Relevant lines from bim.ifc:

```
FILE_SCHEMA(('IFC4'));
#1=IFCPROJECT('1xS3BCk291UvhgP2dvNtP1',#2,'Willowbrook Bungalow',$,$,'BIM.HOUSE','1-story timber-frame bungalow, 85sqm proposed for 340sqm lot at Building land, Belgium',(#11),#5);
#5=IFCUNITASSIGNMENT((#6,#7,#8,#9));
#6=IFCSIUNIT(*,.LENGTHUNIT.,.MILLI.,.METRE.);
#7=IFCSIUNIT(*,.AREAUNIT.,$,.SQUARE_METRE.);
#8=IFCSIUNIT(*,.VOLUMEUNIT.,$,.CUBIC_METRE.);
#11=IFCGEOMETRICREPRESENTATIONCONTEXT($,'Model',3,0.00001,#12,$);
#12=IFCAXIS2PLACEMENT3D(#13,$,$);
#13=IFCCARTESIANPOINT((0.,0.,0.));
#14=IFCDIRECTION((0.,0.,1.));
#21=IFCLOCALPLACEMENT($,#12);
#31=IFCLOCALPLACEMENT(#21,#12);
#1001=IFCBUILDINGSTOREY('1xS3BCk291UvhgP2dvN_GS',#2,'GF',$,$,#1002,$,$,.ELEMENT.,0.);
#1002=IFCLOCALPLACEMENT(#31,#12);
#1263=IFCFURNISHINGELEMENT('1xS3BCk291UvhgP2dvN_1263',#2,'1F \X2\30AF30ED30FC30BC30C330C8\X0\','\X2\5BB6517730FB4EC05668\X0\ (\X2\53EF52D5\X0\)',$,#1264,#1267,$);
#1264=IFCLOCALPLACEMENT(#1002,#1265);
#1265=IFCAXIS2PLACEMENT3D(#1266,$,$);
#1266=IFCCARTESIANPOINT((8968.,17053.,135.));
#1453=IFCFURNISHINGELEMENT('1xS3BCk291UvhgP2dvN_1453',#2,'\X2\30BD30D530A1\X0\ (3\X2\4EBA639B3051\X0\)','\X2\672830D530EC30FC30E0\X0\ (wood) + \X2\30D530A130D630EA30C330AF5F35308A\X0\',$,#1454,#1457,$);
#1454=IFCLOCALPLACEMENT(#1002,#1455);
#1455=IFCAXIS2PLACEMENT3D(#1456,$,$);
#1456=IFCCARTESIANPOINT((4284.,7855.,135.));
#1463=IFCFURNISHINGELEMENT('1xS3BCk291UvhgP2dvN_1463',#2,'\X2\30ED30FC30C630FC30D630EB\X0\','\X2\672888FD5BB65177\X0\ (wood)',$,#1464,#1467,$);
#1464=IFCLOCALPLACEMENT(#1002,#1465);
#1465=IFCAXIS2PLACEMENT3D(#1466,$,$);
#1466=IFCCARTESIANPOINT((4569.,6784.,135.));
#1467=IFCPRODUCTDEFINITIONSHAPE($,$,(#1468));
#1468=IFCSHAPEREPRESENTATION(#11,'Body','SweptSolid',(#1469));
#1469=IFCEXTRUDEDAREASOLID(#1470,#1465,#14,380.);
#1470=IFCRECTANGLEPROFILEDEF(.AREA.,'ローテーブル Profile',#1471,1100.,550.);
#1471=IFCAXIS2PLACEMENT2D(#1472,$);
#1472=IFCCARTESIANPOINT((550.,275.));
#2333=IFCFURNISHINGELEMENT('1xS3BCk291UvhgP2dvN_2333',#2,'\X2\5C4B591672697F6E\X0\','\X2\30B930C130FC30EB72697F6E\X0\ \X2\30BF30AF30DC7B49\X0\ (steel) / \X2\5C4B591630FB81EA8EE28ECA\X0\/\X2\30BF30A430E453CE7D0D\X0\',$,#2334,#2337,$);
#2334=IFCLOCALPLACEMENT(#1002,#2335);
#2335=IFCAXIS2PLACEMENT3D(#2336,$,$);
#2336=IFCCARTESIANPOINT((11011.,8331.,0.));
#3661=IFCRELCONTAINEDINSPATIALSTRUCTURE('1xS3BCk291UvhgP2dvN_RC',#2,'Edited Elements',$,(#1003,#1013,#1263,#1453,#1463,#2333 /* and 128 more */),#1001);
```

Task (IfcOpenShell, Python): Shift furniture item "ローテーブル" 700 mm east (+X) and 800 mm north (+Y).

```python
import ifcopenshell
import ifcopenshell.api.geometry
import ifcopenshell.util.placement
import ifcopenshell.util.unit

model = ifcopenshell.open("bim.ifc")
unit_scale = ifcopenshell.util.unit.calculate_unit_scale(model)

item = model.by_guid("1xS3BCk291UvhgP2dvN_1463")
matrix = ifcopenshell.util.placement.get_local_placement(item.ObjectPlacement)
matrix[0, 3] += 0.7 / unit_scale
matrix[1, 3] += 0.8 / unit_scale
ifcopenshell.api.geometry.edit_object_placement(model, product=item, matrix=matrix, is_si=False)

print(ifcopenshell.util.placement.get_local_placement(item.ObjectPlacement).round(3) + 0.0)

model.write("bim_rev.ifc")
```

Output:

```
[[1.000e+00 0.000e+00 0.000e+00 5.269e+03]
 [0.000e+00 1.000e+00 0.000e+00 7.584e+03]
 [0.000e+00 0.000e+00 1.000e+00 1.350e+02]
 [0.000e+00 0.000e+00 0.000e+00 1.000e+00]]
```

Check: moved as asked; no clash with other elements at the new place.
